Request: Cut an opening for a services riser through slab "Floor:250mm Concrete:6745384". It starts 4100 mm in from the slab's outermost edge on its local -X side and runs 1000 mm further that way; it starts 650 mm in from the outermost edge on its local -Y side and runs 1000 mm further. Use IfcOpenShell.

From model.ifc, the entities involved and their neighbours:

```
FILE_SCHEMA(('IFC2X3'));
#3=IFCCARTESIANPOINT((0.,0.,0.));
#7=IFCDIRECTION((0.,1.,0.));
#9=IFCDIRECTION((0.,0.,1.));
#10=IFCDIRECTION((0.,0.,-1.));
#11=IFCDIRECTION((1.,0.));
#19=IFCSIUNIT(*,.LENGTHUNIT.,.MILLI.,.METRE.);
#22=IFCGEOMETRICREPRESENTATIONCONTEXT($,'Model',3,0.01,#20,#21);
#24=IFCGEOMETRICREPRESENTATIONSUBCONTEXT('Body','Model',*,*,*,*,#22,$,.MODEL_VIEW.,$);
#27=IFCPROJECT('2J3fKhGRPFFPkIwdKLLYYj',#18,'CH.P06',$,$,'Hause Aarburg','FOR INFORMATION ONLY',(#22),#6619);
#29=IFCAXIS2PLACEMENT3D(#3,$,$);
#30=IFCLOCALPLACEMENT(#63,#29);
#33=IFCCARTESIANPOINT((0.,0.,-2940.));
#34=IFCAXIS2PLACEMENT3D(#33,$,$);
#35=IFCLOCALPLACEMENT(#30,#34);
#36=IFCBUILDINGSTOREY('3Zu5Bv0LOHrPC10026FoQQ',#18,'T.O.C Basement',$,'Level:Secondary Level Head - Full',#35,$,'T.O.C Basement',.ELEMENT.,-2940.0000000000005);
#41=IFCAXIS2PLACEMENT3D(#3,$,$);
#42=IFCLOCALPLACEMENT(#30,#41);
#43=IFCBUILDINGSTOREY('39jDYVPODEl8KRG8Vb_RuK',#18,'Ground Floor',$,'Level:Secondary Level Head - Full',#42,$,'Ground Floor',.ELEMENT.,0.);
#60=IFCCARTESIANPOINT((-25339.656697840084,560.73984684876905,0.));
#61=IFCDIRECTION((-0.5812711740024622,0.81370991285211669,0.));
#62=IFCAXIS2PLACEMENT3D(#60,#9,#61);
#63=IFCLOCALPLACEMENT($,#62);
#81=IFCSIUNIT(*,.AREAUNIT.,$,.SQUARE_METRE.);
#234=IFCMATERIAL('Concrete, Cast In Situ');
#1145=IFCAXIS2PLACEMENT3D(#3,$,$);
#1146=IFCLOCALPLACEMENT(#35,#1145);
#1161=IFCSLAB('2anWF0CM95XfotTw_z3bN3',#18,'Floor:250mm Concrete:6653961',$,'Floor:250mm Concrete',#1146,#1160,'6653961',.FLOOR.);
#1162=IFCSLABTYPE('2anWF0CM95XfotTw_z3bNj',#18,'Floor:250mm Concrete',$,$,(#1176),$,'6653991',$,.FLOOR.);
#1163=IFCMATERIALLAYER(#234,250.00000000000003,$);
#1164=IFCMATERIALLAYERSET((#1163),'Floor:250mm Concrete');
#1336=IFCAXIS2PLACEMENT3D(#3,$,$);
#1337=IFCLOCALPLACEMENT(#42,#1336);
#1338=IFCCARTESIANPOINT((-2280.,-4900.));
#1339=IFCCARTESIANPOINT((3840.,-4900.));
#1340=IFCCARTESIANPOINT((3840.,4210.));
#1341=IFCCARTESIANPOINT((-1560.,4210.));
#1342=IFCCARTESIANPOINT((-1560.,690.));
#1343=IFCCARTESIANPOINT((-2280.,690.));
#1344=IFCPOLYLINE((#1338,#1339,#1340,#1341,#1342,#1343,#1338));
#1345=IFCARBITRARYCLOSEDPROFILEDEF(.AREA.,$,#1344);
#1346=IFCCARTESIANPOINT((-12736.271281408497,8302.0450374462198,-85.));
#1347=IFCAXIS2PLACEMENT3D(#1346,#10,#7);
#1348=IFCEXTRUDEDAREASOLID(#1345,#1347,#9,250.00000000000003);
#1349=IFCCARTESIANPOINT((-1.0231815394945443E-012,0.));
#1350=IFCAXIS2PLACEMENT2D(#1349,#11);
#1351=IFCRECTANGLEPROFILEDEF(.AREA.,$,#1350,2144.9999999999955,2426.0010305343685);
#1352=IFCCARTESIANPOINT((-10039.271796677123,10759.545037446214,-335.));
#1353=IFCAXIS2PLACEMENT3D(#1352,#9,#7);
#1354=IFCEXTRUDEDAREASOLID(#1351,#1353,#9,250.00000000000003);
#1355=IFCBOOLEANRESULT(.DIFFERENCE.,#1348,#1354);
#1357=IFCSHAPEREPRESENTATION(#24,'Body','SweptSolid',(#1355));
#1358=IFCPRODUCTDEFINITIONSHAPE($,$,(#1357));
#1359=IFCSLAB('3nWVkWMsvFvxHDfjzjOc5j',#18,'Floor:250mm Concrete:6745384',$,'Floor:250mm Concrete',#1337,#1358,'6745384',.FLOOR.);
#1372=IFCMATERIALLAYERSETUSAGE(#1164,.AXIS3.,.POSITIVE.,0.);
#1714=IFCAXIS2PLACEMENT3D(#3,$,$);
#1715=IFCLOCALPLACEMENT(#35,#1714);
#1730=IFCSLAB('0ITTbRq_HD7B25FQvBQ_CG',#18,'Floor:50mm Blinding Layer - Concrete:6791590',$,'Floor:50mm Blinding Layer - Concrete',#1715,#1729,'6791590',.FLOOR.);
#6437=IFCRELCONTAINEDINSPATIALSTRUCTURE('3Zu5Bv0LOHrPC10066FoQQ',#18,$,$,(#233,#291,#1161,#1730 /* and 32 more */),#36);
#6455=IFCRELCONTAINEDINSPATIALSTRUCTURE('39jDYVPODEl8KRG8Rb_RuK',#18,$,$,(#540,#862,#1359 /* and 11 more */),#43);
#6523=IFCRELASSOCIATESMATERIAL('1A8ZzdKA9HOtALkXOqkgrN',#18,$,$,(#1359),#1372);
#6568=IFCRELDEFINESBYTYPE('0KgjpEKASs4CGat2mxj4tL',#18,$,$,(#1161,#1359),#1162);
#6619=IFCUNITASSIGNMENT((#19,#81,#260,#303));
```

```python
import numpy as np
import ifcopenshell
import ifcopenshell.api.feature
import ifcopenshell.api.geometry
import ifcopenshell.api.root
import ifcopenshell.geom
import ifcopenshell.util.placement
import ifcopenshell.util.representation
import ifcopenshell.util.shape
import ifcopenshell.util.unit

model = ifcopenshell.open("model.ifc")
unit_scale = ifcopenshell.util.unit.calculate_unit_scale(model)
settings = ifcopenshell.geom.settings()


def volume(element):
    """Net volume in cubic metres, openings subtracted."""
    shape = ifcopenshell.geom.create_shape(settings, element)
    return ifcopenshell.util.shape.get_volume(shape.geometry)


slab = model.by_id(1359)
before = volume(slab)

# Extent in the slab's own axes, in metres. The edges named are its -X and -Y sides.
slab_shape = ifcopenshell.geom.create_shape(settings, slab)
vertices = ifcopenshell.util.shape.get_vertices(slab_shape.geometry)
x_min, y_min, bottom = vertices.min(axis=0)
top = vertices[:, 2].max()

opening = ifcopenshell.api.root.create_entity(model, ifc_class="IfcOpeningElement", name="Services riser opening")
context = ifcopenshell.util.representation.get_context(model, "Model", "Body", "MODEL_VIEW")
width, depth = 1, 1
outline = [(0.0, 0.0), (width, 0.0), (width, depth), (0.0, depth), (0.0, 0.0)]
# Overshoot both faces by 50 mm so the cut is clean.
shape = ifcopenshell.api.geometry.add_slab_representation(
    model, context=context, depth=top - bottom + 0.1, polyline=outline
)
ifcopenshell.api.geometry.assign_representation(model, product=opening, representation=shape)

matrix = ifcopenshell.util.placement.get_local_placement(slab.ObjectPlacement)
matrix[:, 3] = matrix @ np.append(np.array([x_min + 4.1, y_min + 0.65, bottom - 0.05]) / unit_scale, 1.0)
ifcopenshell.api.geometry.edit_object_placement(model, product=opening, matrix=matrix, is_si=False)
ifcopenshell.api.feature.add_feature(model, feature=opening, element=slab)

after = volume(slab)

print(f"slab volume {before:.3f} -> {after:.3f} m3")

model.write("model_edited.ifc")
```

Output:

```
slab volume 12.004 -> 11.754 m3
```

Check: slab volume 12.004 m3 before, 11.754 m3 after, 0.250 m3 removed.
